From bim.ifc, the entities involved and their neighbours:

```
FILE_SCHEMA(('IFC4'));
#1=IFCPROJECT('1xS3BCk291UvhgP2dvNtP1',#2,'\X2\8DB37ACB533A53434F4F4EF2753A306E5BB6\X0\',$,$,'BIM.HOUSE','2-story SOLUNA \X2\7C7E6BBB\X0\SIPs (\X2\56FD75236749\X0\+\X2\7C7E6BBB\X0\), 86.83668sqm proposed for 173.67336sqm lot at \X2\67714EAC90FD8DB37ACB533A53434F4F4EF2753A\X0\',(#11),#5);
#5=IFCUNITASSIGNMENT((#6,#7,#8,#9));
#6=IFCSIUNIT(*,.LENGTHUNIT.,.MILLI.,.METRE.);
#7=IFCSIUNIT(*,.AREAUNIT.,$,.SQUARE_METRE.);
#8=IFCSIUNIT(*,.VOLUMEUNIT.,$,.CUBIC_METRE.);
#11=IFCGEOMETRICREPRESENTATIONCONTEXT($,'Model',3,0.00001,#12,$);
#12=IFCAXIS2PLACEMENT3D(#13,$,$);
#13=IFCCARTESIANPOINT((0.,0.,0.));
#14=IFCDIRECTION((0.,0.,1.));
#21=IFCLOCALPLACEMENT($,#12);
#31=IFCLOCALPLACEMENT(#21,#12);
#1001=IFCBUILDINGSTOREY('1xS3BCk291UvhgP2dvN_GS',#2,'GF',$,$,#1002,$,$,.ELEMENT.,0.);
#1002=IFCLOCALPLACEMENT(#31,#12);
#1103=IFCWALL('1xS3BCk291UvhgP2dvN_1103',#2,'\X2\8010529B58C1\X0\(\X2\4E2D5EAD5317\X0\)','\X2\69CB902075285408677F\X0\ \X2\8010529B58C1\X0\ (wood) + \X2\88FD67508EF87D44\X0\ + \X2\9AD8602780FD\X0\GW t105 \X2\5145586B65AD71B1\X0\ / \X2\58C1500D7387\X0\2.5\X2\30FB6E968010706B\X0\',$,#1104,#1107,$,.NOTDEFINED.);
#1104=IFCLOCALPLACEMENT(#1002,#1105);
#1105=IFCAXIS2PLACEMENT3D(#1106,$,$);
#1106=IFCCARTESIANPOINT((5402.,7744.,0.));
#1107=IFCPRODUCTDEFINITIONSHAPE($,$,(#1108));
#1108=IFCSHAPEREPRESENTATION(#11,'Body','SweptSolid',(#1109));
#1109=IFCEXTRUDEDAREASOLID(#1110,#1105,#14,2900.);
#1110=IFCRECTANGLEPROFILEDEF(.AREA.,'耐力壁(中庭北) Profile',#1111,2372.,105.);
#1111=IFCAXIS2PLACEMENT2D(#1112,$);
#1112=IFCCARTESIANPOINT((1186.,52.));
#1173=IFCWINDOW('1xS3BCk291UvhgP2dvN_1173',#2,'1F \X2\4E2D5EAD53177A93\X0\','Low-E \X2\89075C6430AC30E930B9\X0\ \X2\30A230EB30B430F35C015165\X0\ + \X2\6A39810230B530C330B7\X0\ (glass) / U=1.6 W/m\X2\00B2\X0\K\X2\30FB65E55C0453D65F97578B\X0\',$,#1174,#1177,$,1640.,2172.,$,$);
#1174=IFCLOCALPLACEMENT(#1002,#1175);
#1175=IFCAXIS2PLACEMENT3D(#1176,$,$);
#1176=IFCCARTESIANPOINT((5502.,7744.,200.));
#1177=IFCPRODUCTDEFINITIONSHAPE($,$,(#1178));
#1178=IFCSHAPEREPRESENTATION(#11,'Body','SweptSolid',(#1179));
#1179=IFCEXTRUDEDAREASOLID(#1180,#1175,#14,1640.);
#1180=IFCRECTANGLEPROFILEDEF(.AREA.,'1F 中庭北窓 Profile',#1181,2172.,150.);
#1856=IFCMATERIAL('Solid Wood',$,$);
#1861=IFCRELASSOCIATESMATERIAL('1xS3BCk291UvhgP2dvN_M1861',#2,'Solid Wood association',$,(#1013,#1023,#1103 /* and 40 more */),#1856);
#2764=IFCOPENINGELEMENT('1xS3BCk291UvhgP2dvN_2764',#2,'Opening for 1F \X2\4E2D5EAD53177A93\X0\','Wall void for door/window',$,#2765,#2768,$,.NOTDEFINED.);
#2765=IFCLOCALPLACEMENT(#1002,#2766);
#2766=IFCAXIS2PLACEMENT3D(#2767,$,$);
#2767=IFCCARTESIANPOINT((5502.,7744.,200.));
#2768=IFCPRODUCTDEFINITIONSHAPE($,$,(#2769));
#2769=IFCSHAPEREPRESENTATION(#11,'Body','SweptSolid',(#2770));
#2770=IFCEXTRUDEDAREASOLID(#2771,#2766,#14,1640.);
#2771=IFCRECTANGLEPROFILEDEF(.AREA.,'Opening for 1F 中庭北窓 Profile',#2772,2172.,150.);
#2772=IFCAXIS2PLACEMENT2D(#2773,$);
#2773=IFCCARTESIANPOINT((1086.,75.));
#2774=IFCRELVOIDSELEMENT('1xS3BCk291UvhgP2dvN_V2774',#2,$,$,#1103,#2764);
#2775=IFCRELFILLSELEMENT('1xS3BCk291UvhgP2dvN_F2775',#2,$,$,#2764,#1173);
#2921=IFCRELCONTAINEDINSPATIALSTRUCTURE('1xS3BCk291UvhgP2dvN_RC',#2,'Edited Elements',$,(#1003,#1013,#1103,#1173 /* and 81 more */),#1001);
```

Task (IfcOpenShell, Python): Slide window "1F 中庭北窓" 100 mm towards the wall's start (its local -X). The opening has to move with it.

```python
import ifcopenshell
import ifcopenshell.api.geometry
import ifcopenshell.util.placement
import ifcopenshell.util.unit

model = ifcopenshell.open("bim.ifc")
unit_scale = ifcopenshell.util.unit.calculate_unit_scale(model)

window = model.by_guid("1xS3BCk291UvhgP2dvN_1173")
opening = window.FillsVoids[0].RelatingOpeningElement
wall = opening.VoidsElements[0].RelatingBuildingElement

wall_matrix = ifcopenshell.util.placement.get_local_placement(wall.ObjectPlacement)
shift = wall_matrix[:3, 0] * -0.1 / unit_scale
before = ifcopenshell.util.placement.get_local_placement(window.ObjectPlacement)[:3, 3].copy()

# The window is not placed relative to its opening, so move both.
for product in (opening, window):
    matrix = ifcopenshell.util.placement.get_local_placement(product.ObjectPlacement)
    matrix[:3, 3] += shift
    ifcopenshell.api.geometry.edit_object_placement(model, product=product, matrix=matrix, is_si=False)

after = ifcopenshell.util.placement.get_local_placement(window.ObjectPlacement)[:3, 3]
print("window moved by", (after - before).round(3) + 0.0)

model.write("bim_rev.ifc")
```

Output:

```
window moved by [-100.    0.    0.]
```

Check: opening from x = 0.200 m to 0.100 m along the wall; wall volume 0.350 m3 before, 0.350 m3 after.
